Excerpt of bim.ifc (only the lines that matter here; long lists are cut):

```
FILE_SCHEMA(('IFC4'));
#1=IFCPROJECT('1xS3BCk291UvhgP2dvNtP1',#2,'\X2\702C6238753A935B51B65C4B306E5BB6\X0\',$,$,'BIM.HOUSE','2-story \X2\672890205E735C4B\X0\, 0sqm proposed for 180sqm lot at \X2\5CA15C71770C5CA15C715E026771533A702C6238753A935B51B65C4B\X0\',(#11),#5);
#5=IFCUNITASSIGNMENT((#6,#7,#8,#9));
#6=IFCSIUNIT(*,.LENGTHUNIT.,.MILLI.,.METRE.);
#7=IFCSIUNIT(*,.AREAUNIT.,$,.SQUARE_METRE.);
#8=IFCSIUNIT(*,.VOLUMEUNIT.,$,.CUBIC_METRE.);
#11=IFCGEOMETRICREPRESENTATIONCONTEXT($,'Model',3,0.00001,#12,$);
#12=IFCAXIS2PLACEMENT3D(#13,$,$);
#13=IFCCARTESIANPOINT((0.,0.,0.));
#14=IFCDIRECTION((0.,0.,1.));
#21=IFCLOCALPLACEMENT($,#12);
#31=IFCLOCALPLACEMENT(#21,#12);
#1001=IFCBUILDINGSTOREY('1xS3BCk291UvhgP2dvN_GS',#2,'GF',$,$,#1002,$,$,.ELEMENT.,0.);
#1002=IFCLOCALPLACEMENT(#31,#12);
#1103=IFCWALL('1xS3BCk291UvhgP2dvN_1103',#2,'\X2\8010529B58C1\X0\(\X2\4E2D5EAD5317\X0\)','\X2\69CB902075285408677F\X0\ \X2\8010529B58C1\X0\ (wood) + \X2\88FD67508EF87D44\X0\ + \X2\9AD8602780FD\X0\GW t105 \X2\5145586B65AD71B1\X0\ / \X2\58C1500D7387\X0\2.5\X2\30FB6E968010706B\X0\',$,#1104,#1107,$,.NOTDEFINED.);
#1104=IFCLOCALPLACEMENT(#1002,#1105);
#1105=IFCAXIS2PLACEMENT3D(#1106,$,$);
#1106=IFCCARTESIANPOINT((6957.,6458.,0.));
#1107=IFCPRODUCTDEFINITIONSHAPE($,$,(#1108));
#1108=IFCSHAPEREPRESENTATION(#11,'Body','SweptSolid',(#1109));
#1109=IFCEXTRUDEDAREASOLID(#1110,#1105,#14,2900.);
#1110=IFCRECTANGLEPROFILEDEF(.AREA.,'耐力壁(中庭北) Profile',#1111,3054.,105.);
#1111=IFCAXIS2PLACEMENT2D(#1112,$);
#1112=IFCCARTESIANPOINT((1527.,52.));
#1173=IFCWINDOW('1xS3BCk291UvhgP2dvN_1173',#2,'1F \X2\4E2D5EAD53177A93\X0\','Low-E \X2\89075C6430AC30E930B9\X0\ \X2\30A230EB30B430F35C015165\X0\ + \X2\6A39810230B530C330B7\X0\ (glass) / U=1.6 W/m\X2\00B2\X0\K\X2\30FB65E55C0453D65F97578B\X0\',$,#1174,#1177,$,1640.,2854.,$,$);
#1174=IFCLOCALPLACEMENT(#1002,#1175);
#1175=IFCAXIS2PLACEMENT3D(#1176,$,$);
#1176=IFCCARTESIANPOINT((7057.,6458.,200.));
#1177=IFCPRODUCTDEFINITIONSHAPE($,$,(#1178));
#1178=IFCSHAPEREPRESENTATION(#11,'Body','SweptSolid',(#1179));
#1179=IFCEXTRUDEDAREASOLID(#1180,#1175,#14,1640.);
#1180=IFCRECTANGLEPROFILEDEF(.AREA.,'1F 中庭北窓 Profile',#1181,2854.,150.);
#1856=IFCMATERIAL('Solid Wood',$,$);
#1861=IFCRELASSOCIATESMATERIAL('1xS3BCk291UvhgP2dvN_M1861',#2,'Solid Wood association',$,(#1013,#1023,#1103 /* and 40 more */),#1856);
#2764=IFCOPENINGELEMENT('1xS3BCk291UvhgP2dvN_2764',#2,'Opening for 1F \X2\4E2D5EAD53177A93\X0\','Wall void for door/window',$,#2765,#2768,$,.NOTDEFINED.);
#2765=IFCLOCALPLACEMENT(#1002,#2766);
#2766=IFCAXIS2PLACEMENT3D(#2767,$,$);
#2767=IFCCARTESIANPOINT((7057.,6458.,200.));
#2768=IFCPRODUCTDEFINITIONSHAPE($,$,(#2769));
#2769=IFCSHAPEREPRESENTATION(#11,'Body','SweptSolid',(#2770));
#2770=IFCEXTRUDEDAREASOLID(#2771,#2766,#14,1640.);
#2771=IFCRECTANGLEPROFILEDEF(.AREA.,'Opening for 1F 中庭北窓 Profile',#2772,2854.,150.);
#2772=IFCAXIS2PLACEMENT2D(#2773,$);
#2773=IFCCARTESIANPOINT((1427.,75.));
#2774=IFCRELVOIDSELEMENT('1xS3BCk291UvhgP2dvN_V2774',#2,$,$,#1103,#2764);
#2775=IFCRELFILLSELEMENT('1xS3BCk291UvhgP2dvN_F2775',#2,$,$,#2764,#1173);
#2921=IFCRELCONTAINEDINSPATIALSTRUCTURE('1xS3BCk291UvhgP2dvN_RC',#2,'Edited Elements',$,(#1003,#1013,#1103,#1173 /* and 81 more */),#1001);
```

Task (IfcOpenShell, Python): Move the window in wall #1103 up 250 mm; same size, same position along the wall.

```python
import numpy as np
import ifcopenshell
import ifcopenshell.api.geometry
import ifcopenshell.util.placement
import ifcopenshell.util.unit

model = ifcopenshell.open("bim.ifc")
unit_scale = ifcopenshell.util.unit.calculate_unit_scale(model)

window = model.by_id(1173)
opening = window.FillsVoids[0].RelatingOpeningElement
dz = 250.0

shift = np.array([0.0, 0.0, dz])
# The window is not placed relative to its opening, so move both.
for product in (opening, window):
    matrix = ifcopenshell.util.placement.get_local_placement(product.ObjectPlacement)
    matrix[:3, 3] += shift
    ifcopenshell.api.geometry.edit_object_placement(model, product=product, matrix=matrix, is_si=False)

print(f"moved by {dz * unit_scale:+.3f} m")

model.write("bim_rev.ifc")
```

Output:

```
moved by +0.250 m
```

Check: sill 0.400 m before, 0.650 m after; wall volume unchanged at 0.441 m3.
